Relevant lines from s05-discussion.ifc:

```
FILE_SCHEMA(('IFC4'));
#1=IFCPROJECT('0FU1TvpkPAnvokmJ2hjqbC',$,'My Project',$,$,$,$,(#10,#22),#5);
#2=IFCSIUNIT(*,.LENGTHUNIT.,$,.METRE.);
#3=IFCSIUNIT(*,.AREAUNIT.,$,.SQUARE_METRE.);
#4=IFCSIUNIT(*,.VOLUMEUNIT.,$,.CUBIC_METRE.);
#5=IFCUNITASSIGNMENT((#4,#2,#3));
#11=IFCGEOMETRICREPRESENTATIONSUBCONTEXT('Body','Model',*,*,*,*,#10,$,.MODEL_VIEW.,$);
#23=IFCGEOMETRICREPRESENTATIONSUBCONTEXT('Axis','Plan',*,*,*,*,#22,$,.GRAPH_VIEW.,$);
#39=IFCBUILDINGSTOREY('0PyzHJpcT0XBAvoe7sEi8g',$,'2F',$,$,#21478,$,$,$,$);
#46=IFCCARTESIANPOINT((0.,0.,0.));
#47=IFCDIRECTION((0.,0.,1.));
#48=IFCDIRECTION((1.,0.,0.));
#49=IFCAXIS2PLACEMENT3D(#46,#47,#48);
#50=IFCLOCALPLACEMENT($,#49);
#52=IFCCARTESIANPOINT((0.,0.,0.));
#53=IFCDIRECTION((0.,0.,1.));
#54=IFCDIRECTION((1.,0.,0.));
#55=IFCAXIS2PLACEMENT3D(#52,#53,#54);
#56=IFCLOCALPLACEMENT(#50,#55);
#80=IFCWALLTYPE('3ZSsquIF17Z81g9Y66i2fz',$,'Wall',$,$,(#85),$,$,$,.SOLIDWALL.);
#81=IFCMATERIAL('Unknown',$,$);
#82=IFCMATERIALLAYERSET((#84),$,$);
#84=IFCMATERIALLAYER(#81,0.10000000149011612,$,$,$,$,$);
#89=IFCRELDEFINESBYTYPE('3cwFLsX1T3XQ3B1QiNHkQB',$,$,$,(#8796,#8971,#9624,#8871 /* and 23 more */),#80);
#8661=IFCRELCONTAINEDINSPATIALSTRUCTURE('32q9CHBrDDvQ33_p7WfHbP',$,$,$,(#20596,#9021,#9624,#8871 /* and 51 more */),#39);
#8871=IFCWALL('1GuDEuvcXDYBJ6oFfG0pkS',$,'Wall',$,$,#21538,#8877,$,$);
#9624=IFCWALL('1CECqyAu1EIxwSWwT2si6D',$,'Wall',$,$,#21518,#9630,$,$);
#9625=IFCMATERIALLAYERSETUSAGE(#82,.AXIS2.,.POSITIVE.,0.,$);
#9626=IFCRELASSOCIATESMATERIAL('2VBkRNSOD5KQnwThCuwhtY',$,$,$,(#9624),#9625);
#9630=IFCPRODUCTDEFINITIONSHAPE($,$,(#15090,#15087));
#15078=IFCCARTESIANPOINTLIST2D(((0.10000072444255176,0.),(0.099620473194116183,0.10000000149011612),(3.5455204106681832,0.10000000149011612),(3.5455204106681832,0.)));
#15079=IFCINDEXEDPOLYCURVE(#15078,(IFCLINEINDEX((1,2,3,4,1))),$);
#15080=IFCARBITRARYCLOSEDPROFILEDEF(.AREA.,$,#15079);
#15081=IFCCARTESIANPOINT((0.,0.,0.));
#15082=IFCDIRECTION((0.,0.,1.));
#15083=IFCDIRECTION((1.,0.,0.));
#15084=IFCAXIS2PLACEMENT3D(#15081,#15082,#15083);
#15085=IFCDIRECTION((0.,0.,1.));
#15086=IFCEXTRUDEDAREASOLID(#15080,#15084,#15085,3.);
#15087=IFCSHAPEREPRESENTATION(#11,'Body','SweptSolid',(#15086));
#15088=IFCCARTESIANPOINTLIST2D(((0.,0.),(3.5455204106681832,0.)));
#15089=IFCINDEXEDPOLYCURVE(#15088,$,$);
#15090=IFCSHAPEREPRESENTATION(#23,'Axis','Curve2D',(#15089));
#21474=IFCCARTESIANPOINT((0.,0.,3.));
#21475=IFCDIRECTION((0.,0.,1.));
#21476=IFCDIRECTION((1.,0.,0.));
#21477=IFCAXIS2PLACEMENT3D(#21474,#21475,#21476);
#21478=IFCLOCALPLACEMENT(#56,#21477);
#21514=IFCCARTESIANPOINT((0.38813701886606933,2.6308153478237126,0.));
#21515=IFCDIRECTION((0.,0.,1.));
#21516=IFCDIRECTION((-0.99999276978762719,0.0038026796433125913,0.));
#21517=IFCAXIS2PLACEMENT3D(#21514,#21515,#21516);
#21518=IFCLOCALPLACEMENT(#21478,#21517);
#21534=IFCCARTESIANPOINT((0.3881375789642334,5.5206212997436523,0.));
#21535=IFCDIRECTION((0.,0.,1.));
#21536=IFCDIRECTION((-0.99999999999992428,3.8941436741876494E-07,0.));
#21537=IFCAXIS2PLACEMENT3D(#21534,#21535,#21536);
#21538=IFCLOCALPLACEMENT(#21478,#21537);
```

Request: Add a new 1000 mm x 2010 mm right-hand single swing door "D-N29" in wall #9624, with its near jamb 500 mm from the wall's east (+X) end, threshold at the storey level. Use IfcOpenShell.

```python
import numpy as np
import ifcopenshell
import ifcopenshell.api.feature
import ifcopenshell.api.geometry
import ifcopenshell.api.root
import ifcopenshell.api.spatial
import ifcopenshell.geom
import ifcopenshell.util.element
import ifcopenshell.util.placement
import ifcopenshell.util.representation
import ifcopenshell.util.shape
import ifcopenshell.util.unit

model = ifcopenshell.open("s05-discussion.ifc")
unit_scale = ifcopenshell.util.unit.calculate_unit_scale(model)
settings = ifcopenshell.geom.settings()


def volume(element):
    """Net volume in cubic metres, openings subtracted."""
    shape = ifcopenshell.geom.create_shape(settings, element)
    return ifcopenshell.util.shape.get_volume(shape.geometry)


wall = model.by_id(9624)
storey = ifcopenshell.util.element.get_container(wall, ifc_class="IfcBuildingStorey")
context = ifcopenshell.util.representation.get_context(model, "Model", "Body", "MODEL_VIEW")
before = volume(wall)

width, height, from_end, sill = 1, 2.01, 0.5, 0.0  # metres

# The wall runs along its own X axis, and the end named is its -X end.
wall_shape = ifcopenshell.geom.create_shape(settings, wall)
x, y, z = ifcopenshell.util.shape.get_vertices(wall_shape.geometry).T
start = x.min() + from_end
face, thickness = float(y.min()), float(y.max() - y.min())
wall_matrix = ifcopenshell.util.placement.get_local_placement(wall.ObjectPlacement)
level = ifcopenshell.util.placement.get_local_placement(storey.ObjectPlacement)[2, 3]


def in_wall(x, y):
    """Placement at x, y metres in the wall's axes, at sill height."""
    matrix = wall_matrix.copy()
    matrix[:, 3] = wall_matrix @ np.array([x / unit_scale, y / unit_scale, 0.0, 1.0])
    matrix[2, 3] = level + sill / unit_scale
    return matrix


# Opening: a box that overshoots both wall faces by 50 mm.
opening = ifcopenshell.api.root.create_entity(model, ifc_class="IfcOpeningElement", predefined_type="OPENING")
box = ifcopenshell.api.geometry.add_wall_representation(
    model, context=context, length=width, height=height, thickness=thickness + 0.1
)
ifcopenshell.api.geometry.assign_representation(model, product=opening, representation=box)
ifcopenshell.api.geometry.edit_object_placement(model, product=opening, matrix=in_wall(start, face - 0.05), is_si=False)
ifcopenshell.api.feature.add_feature(model, feature=opening, element=wall)

door = ifcopenshell.api.root.create_entity(model, ifc_class="IfcDoor", name="D-N29", predefined_type="DOOR")
door.OverallWidth, door.OverallHeight = width / unit_scale, height / unit_scale
door.OperationType = "SINGLE_SWING_RIGHT"
body = ifcopenshell.api.geometry.add_door_representation(
    model,
    context=context,
    overall_width=door.OverallWidth,
    overall_height=door.OverallHeight,
    operation_type="SINGLE_SWING_RIGHT",
    lining_properties={"LiningDepth": thickness / unit_scale, "ThresholdDepth": thickness / unit_scale},
)
ifcopenshell.api.geometry.assign_representation(model, product=door, representation=body)
ifcopenshell.api.spatial.assign_container(model, products=[door], relating_structure=storey)
ifcopenshell.api.feature.add_filling(model, opening=opening, element=door)

# The lining spans the wall, so the door starts at the wall face.
ifcopenshell.api.geometry.edit_object_placement(model, product=door, matrix=in_wall(start, face), is_si=False)

after = volume(wall)

print(f"wall volume {before:.3f} -> {after:.3f} m3")

model.write("s05-discussion_edited.ifc")
```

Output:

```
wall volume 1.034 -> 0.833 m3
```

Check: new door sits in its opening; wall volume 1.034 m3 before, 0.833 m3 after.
